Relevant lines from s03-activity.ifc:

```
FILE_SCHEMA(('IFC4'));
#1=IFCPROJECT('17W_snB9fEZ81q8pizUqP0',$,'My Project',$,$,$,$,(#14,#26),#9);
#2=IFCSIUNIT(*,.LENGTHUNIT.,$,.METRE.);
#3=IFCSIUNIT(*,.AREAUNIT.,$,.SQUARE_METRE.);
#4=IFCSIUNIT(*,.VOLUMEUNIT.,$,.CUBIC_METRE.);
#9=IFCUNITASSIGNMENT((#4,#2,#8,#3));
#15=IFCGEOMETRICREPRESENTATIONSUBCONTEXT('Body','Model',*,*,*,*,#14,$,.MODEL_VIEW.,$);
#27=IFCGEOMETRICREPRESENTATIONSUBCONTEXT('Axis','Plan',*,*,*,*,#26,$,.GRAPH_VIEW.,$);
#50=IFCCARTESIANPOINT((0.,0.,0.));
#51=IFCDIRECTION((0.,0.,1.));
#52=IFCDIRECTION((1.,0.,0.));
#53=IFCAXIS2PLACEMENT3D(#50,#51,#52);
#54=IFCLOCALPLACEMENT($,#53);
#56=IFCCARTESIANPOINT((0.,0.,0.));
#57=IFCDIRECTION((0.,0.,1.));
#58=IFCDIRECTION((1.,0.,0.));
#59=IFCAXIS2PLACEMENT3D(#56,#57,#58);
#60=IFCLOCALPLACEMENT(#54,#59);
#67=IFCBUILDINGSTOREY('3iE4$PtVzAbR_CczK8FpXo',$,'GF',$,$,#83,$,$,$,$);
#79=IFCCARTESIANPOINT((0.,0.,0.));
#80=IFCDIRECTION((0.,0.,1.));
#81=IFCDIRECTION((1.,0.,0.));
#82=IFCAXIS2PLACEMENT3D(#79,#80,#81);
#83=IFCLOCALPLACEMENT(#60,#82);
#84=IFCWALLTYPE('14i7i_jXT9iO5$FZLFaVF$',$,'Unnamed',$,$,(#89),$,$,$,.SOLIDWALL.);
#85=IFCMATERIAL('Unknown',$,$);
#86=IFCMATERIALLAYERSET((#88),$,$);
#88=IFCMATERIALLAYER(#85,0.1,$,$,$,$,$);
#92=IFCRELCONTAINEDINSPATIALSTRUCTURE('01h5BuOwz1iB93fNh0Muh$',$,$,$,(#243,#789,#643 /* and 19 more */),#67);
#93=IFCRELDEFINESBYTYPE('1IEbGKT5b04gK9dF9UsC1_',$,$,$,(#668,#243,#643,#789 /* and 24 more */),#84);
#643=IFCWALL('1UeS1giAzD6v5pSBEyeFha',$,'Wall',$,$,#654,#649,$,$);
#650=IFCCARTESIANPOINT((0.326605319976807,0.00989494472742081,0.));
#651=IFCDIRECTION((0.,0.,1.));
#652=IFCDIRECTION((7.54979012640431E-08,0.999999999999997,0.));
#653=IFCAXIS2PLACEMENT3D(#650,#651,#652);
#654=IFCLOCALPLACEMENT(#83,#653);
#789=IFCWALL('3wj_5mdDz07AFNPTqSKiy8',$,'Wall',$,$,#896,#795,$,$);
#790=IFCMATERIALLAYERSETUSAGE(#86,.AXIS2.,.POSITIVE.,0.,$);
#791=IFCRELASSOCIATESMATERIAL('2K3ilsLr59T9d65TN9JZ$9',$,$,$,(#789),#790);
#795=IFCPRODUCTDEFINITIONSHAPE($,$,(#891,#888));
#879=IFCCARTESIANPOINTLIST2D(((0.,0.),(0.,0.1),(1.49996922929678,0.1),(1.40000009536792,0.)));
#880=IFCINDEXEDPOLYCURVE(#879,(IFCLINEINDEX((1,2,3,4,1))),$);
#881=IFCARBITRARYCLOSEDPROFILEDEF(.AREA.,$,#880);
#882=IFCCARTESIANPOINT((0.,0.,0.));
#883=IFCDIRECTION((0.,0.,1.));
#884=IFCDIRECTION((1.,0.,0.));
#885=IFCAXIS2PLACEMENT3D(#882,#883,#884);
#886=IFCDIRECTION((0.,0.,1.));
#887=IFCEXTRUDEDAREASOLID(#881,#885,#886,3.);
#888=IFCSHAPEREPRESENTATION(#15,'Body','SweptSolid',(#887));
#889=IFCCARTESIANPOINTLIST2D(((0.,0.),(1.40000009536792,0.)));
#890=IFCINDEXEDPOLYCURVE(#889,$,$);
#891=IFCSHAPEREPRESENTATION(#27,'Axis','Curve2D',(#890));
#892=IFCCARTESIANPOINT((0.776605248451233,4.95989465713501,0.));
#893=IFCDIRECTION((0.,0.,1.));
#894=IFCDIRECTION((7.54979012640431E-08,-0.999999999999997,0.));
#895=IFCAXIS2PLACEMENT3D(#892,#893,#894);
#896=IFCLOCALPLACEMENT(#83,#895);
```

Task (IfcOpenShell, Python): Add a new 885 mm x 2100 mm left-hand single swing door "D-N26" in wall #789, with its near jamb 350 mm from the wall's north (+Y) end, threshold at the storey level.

```python
import numpy as np
import ifcopenshell
import ifcopenshell.api.feature
import ifcopenshell.api.geometry
import ifcopenshell.api.root
import ifcopenshell.api.spatial
import ifcopenshell.geom
import ifcopenshell.util.element
import ifcopenshell.util.placement
import ifcopenshell.util.representation
import ifcopenshell.util.shape
import ifcopenshell.util.unit

model = ifcopenshell.open("s03-activity.ifc")
unit_scale = ifcopenshell.util.unit.calculate_unit_scale(model)
settings = ifcopenshell.geom.settings()


def volume(element):
    """Net volume in cubic metres, openings subtracted."""
    shape = ifcopenshell.geom.create_shape(settings, element)
    return ifcopenshell.util.shape.get_volume(shape.geometry)


wall = model.by_guid("3wj_5mdDz07AFNPTqSKiy8")
storey = ifcopenshell.util.element.get_container(wall, ifc_class="IfcBuildingStorey")
context = ifcopenshell.util.representation.get_context(model, "Model", "Body", "MODEL_VIEW")
before = volume(wall)

width, height, from_end, sill = 0.885, 2.1, 0.35, 0.0  # metres

# The wall runs along its own X axis, and the end named is its -X end.
wall_shape = ifcopenshell.geom.create_shape(settings, wall)
x, y, z = ifcopenshell.util.shape.get_vertices(wall_shape.geometry).T
start = x.min() + from_end
face, thickness = float(y.min()), float(y.max() - y.min())
wall_matrix = ifcopenshell.util.placement.get_local_placement(wall.ObjectPlacement)
level = ifcopenshell.util.placement.get_local_placement(storey.ObjectPlacement)[2, 3]


def in_wall(x, y):
    """Placement at x, y metres in the wall's axes, at sill height."""
    matrix = wall_matrix.copy()
    matrix[:, 3] = wall_matrix @ np.array([x / unit_scale, y / unit_scale, 0.0, 1.0])
    matrix[2, 3] = level + sill / unit_scale
    return matrix


# Opening: a box that overshoots both wall faces by 50 mm.
opening = ifcopenshell.api.root.create_entity(model, ifc_class="IfcOpeningElement", predefined_type="OPENING")
box = ifcopenshell.api.geometry.add_wall_representation(
    model, context=context, length=width, height=height, thickness=thickness + 0.1
)
ifcopenshell.api.geometry.assign_representation(model, product=opening, representation=box)
ifcopenshell.api.geometry.edit_object_placement(model, product=opening, matrix=in_wall(start, face - 0.05), is_si=False)
ifcopenshell.api.feature.add_feature(model, feature=opening, element=wall)

door = ifcopenshell.api.root.create_entity(model, ifc_class="IfcDoor", name="D-N26", predefined_type="DOOR")
door.OverallWidth, door.OverallHeight = width / unit_scale, height / unit_scale
door.OperationType = "SINGLE_SWING_LEFT"
body = ifcopenshell.api.geometry.add_door_representation(
    model,
    context=context,
    overall_width=door.OverallWidth,
    overall_height=door.OverallHeight,
    operation_type="SINGLE_SWING_LEFT",
    lining_properties={"LiningDepth": thickness / unit_scale, "ThresholdDepth": thickness / unit_scale},
)
ifcopenshell.api.geometry.assign_representation(model, product=door, representation=body)
ifcopenshell.api.spatial.assign_container(model, products=[door], relating_structure=storey)
ifcopenshell.api.feature.add_filling(model, opening=opening, element=door)

# The lining spans the wall, so the door starts at the wall face.
ifcopenshell.api.geometry.edit_object_placement(model, product=door, matrix=in_wall(start, face), is_si=False)

after = volume(wall)

print(f"wall volume {before:.3f} -> {after:.3f} m3")

model.write("s03-activity_rev.ifc")
```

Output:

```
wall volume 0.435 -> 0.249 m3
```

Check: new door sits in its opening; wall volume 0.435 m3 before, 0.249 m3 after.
